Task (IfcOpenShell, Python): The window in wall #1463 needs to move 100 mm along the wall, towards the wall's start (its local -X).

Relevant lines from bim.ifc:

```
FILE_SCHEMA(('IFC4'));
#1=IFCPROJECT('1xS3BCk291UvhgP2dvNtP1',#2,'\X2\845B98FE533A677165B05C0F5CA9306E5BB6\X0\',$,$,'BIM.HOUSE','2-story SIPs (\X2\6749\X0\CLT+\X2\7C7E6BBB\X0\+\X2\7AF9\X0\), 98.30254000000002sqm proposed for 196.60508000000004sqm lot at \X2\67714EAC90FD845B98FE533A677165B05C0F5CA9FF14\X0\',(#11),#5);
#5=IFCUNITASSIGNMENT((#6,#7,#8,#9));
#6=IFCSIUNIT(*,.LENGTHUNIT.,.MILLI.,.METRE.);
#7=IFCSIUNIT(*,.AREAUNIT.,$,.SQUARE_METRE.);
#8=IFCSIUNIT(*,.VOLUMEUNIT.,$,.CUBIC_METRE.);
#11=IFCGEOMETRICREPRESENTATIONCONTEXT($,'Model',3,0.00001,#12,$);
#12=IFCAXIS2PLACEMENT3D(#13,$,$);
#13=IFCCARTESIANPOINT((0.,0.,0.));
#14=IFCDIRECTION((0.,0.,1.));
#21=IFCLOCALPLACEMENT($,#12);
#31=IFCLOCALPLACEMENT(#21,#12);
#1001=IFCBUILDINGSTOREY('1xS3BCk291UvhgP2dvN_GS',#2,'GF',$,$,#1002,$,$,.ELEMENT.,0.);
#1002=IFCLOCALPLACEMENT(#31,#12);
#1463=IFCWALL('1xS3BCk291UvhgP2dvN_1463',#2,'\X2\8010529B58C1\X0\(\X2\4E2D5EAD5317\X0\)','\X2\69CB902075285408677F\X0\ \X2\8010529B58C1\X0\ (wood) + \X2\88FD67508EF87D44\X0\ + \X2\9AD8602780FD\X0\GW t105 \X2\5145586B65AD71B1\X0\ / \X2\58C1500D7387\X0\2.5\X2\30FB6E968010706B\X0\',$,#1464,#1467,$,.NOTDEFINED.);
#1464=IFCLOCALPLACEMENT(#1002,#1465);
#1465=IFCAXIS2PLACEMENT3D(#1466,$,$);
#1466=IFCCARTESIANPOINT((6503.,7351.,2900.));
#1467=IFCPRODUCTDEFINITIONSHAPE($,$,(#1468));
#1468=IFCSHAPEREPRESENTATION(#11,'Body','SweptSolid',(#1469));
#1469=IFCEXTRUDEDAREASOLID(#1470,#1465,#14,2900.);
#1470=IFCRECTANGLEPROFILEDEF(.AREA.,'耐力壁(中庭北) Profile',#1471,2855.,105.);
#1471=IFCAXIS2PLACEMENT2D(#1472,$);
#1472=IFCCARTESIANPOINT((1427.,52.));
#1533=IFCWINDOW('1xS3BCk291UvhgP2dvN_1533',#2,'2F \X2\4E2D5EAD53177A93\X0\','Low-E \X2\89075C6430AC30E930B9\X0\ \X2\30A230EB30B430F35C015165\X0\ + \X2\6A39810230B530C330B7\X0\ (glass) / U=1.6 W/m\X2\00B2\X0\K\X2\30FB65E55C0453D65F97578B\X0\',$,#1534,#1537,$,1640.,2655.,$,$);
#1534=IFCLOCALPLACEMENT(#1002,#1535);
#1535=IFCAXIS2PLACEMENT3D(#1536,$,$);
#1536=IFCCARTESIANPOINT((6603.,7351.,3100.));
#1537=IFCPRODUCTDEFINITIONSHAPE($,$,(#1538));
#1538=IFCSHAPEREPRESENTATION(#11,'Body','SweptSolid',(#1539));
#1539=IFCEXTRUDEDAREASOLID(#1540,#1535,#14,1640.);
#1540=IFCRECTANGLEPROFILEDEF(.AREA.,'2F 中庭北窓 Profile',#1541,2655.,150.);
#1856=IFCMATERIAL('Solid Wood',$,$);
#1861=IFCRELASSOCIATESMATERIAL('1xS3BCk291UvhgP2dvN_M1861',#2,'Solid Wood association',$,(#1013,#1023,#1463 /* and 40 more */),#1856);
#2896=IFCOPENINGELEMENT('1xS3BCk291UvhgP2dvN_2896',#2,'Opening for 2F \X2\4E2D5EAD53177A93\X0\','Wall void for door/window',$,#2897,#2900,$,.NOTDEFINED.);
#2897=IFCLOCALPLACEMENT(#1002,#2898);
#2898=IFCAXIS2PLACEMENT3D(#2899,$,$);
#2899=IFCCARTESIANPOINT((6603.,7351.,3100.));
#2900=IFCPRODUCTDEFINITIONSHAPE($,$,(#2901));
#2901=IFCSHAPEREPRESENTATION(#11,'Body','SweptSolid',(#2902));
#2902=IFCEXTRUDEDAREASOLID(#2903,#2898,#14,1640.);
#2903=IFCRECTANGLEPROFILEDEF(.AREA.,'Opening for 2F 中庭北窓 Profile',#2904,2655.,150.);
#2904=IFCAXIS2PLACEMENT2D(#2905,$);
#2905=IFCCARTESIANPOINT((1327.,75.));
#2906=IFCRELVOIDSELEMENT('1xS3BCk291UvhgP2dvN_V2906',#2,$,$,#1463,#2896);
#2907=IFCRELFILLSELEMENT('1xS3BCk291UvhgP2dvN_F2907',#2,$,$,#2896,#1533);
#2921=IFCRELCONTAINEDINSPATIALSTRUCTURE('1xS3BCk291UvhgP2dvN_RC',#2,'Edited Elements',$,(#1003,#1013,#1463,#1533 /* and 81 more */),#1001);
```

```python
import ifcopenshell
import ifcopenshell.api.geometry
import ifcopenshell.util.placement
import ifcopenshell.util.unit

model = ifcopenshell.open("bim.ifc")
unit_scale = ifcopenshell.util.unit.calculate_unit_scale(model)

window = model.by_guid("1xS3BCk291UvhgP2dvN_1533")
opening = window.FillsVoids[0].RelatingOpeningElement
wall = opening.VoidsElements[0].RelatingBuildingElement

wall_matrix = ifcopenshell.util.placement.get_local_placement(wall.ObjectPlacement)
shift = wall_matrix[:3, 0] * -0.1 / unit_scale
before = ifcopenshell.util.placement.get_local_placement(window.ObjectPlacement)[:3, 3].copy()

# The window is not placed relative to its opening, so move both.
for product in (opening, window):
    matrix = ifcopenshell.util.placement.get_local_placement(product.ObjectPlacement)
    matrix[:3, 3] += shift
    ifcopenshell.api.geometry.edit_object_placement(model, product=product, matrix=matrix, is_si=False)

after = ifcopenshell.util.placement.get_local_placement(window.ObjectPlacement)[:3, 3]
print("window moved by", (after - before).round(3) + 0.0)

model.write("bim_edited.ifc")
```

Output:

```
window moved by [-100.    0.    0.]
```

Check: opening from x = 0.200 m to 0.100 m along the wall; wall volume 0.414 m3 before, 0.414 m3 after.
